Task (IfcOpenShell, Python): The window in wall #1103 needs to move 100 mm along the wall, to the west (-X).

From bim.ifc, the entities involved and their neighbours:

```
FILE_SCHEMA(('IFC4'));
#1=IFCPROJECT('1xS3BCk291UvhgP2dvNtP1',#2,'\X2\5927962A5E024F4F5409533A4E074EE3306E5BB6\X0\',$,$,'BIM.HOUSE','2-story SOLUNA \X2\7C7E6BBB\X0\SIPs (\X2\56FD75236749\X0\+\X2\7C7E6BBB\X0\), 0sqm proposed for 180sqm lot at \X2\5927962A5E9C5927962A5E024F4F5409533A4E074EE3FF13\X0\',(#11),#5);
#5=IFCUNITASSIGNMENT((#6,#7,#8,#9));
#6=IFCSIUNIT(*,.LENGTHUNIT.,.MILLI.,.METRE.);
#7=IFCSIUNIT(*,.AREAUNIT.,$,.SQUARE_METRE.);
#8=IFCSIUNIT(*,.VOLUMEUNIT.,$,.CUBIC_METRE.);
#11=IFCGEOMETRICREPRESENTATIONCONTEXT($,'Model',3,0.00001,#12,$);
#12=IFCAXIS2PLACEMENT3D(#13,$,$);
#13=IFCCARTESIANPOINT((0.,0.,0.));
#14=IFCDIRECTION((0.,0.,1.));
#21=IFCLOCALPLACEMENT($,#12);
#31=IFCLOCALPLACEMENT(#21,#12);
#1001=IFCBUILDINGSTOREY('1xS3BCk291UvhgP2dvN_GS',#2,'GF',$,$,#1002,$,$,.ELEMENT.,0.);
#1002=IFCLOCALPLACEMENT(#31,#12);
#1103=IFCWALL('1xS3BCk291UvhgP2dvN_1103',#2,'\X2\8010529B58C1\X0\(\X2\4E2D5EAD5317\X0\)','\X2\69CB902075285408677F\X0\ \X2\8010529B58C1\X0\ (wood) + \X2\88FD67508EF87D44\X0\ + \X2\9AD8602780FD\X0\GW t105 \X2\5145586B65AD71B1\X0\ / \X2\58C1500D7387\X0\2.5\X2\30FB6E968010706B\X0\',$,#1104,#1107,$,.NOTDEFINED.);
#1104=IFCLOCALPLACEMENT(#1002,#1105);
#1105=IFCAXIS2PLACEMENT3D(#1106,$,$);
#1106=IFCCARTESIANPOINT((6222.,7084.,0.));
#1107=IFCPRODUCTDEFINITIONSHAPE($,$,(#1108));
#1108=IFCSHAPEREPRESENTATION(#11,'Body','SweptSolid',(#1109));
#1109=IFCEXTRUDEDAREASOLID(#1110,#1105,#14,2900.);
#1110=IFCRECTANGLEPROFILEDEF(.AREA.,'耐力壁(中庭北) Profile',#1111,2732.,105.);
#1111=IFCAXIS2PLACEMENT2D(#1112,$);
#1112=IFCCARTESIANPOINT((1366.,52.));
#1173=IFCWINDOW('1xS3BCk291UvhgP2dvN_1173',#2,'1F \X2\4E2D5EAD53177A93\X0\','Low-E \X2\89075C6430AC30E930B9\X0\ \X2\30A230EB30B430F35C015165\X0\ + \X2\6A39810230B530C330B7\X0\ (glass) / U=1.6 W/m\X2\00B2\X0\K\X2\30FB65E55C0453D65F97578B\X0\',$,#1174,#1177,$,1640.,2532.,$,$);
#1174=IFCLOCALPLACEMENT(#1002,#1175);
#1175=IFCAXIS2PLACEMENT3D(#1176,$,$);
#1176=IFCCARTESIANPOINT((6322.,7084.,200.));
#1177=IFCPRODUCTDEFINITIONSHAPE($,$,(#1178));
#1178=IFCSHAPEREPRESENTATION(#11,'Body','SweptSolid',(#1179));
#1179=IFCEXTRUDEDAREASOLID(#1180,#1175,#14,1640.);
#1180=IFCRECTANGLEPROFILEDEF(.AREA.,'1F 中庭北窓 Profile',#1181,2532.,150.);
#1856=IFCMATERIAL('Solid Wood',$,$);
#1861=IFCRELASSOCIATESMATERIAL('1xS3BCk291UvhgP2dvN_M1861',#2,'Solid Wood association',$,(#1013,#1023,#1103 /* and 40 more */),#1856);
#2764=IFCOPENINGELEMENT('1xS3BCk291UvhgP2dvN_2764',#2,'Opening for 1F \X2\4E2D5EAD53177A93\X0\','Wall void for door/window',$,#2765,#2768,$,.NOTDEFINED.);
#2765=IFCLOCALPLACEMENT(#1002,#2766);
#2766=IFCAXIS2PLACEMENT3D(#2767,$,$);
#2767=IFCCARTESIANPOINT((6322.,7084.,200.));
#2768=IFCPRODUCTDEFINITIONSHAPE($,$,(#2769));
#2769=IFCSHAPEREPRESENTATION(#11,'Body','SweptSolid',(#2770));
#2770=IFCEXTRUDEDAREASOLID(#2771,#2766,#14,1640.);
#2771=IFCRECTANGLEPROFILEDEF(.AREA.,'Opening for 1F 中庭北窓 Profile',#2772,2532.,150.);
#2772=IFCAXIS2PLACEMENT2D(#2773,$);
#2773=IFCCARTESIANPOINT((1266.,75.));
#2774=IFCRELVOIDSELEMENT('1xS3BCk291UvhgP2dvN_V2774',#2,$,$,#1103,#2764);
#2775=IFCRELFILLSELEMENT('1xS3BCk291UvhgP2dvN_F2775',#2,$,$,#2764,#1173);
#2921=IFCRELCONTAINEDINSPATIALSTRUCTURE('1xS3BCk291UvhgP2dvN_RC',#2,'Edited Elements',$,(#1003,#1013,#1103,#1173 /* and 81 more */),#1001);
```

```python
import ifcopenshell
import ifcopenshell.api.geometry
import ifcopenshell.util.placement
import ifcopenshell.util.unit

model = ifcopenshell.open("bim.ifc")
unit_scale = ifcopenshell.util.unit.calculate_unit_scale(model)

window = model.by_guid("1xS3BCk291UvhgP2dvN_1173")
opening = window.FillsVoids[0].RelatingOpeningElement
wall = opening.VoidsElements[0].RelatingBuildingElement

wall_matrix = ifcopenshell.util.placement.get_local_placement(wall.ObjectPlacement)
shift = wall_matrix[:3, 0] * -0.1 / unit_scale
before = ifcopenshell.util.placement.get_local_placement(window.ObjectPlacement)[:3, 3].copy()

# The window is not placed relative to its opening, so move both.
for product in (opening, window):
    matrix = ifcopenshell.util.placement.get_local_placement(product.ObjectPlacement)
    matrix[:3, 3] += shift
    ifcopenshell.api.geometry.edit_object_placement(model, product=product, matrix=matrix, is_si=False)

after = ifcopenshell.util.placement.get_local_placement(window.ObjectPlacement)[:3, 3]
print("window moved by", (after - before).round(3) + 0.0)

model.write("bim_edited.ifc")
```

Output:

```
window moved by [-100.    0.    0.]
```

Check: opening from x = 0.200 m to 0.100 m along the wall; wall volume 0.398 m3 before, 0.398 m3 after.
